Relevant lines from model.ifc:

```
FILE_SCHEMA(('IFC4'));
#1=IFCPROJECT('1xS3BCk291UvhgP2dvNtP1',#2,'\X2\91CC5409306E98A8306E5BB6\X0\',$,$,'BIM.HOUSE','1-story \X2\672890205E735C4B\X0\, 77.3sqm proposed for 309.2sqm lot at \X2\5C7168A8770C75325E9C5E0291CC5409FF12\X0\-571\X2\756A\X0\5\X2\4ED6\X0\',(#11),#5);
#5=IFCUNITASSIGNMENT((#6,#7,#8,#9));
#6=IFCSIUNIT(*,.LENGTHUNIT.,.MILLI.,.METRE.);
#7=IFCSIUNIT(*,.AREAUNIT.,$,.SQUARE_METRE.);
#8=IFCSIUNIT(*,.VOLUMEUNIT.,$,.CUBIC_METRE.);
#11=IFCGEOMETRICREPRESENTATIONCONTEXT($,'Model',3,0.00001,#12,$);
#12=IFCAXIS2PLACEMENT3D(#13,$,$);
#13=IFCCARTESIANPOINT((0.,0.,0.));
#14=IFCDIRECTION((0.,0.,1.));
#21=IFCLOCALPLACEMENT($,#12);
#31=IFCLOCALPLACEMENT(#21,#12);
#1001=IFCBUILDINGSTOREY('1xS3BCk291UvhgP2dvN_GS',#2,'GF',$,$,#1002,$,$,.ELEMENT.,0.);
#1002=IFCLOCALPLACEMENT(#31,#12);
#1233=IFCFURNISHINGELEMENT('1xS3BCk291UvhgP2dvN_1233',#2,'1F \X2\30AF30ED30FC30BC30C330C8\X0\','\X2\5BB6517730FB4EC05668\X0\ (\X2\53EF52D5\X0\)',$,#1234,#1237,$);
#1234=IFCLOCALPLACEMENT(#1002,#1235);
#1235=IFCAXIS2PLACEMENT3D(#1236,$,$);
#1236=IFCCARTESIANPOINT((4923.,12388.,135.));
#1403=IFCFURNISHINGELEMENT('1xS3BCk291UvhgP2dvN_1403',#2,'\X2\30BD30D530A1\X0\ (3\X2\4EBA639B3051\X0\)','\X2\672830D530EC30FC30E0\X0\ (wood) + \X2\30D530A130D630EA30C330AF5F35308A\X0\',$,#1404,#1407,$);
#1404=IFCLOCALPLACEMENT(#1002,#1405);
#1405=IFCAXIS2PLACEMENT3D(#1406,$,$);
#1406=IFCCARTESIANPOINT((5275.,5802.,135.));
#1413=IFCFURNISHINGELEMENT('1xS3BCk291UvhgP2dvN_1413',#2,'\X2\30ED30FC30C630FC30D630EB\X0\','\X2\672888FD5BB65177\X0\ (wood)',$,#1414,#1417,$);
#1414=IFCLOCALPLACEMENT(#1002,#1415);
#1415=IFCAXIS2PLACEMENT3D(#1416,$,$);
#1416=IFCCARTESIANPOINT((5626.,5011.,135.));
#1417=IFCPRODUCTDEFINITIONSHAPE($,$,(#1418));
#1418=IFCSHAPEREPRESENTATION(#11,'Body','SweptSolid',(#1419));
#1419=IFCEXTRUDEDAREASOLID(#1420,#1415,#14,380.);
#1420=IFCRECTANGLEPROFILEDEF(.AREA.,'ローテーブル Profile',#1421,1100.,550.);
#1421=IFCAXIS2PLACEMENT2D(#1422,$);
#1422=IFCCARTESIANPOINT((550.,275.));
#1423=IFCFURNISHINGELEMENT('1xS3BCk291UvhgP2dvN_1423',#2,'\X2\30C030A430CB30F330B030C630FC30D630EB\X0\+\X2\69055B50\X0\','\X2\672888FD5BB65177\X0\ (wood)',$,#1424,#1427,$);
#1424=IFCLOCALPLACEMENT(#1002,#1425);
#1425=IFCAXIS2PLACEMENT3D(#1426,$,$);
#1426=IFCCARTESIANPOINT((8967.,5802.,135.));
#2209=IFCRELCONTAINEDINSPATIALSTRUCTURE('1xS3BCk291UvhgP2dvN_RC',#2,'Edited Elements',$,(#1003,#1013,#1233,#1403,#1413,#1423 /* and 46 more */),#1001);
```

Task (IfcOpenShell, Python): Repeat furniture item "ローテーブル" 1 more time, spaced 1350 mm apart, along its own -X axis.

```python
import ifcopenshell
import ifcopenshell.api.geometry
import ifcopenshell.api.root
import ifcopenshell.util.element
import ifcopenshell.util.placement

model = ifcopenshell.open("model.ifc")


def reuse_history(source, copy):
    """copy_class also copies each property set's owner history, people and application; keep the originals."""
    for rel in copy.IsDefinedBy:
        if rel.is_a("IfcRelDefinesByProperties") and (history := rel.RelatingPropertyDefinition.OwnerHistory):
            rel.RelatingPropertyDefinition.OwnerHistory = source.OwnerHistory
            ifcopenshell.util.element.remove_deep2(model, history)


source = model.by_guid("1xS3BCk291UvhgP2dvN_1413")
base = ifcopenshell.util.placement.get_local_placement(source.ObjectPlacement)
step = -base[:3, 0] * 1350.0

for i in range(1, 2):
    copy = ifcopenshell.api.root.copy_class(model, product=source)
    copy.Representation = ifcopenshell.util.element.copy_deep(
        model, source.Representation, exclude=["IfcGeometricRepresentationContext", "IfcRepresentationMap"]
    )
    reuse_history(source, copy)
    matrix = base.copy()
    matrix[:3, 3] += i * step
    print("added at", matrix[:3, 3].round(3) + 0.0)
    ifcopenshell.api.geometry.edit_object_placement(model, product=copy, matrix=matrix, is_si=False)

model.write("model_rev.ifc")
```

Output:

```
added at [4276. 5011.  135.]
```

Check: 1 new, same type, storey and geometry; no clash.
